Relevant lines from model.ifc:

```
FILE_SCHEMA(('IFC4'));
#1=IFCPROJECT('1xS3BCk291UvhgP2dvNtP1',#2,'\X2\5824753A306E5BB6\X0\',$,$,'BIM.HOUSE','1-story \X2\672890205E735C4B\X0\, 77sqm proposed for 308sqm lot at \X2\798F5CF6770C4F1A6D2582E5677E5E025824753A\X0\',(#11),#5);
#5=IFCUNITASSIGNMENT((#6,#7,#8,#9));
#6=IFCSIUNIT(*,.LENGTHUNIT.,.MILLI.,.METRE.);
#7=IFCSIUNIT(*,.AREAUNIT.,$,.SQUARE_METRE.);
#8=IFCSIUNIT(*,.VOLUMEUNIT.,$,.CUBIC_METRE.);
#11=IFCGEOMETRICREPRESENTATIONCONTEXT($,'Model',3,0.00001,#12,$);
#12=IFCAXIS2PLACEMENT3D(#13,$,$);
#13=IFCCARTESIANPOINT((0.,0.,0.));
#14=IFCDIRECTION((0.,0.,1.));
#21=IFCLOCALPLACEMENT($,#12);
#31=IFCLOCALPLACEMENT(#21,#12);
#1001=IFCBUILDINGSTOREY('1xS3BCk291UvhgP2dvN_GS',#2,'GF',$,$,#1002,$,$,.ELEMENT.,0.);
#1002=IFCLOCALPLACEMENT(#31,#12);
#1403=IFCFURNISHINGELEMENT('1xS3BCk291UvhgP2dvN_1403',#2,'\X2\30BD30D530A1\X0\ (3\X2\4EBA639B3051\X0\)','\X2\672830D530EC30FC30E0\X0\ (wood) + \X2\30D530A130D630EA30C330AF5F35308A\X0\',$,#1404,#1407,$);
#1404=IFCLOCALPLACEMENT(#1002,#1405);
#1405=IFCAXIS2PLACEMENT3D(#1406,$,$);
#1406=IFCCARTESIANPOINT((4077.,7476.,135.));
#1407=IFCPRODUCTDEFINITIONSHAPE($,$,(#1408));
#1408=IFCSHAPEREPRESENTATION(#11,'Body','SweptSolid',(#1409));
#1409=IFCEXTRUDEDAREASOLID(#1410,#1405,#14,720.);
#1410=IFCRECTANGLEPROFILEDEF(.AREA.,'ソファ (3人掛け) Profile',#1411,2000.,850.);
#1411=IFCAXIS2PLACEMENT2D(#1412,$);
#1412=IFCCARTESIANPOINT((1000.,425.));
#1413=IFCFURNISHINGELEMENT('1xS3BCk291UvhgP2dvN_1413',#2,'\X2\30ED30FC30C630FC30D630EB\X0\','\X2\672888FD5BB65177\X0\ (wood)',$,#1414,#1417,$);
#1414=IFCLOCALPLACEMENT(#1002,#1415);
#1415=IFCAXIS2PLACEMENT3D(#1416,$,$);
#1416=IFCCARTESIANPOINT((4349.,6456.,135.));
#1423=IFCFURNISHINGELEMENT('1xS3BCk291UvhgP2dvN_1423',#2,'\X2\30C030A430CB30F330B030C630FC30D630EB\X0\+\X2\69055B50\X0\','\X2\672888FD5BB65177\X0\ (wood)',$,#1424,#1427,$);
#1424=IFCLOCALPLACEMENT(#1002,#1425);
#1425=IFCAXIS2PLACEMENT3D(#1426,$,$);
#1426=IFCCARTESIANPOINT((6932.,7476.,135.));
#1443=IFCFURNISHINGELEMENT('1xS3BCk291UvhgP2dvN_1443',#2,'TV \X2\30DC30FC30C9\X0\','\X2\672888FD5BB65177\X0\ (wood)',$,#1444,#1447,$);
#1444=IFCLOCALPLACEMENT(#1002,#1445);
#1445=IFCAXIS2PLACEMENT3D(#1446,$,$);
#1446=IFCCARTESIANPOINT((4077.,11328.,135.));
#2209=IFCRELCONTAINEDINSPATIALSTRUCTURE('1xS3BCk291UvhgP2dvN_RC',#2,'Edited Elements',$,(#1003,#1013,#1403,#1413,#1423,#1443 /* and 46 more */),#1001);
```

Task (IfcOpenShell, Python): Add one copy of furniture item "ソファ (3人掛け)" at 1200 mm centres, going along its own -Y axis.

```python
import ifcopenshell
import ifcopenshell.api.geometry
import ifcopenshell.api.root
import ifcopenshell.util.element
import ifcopenshell.util.placement
import ifcopenshell.util.unit

model = ifcopenshell.open("model.ifc")
unit_scale = ifcopenshell.util.unit.calculate_unit_scale(model)


def reuse_history(source, copy):
    """copy_class also copies each property set's owner history, people and application; keep the originals."""
    for rel in copy.IsDefinedBy:
        if rel.is_a("IfcRelDefinesByProperties") and (history := rel.RelatingPropertyDefinition.OwnerHistory):
            rel.RelatingPropertyDefinition.OwnerHistory = source.OwnerHistory
            ifcopenshell.util.element.remove_deep2(model, history)


source = model.by_id(1403)
base = ifcopenshell.util.placement.get_local_placement(source.ObjectPlacement)
step = -base[:3, 1] * 1.2 / unit_scale

for i in range(1, 2):
    copy = ifcopenshell.api.root.copy_class(model, product=source)
    copy.Representation = ifcopenshell.util.element.copy_deep(
        model, source.Representation, exclude=["IfcGeometricRepresentationContext", "IfcRepresentationMap"]
    )
    reuse_history(source, copy)
    matrix = base.copy()
    matrix[:3, 3] += i * step
    print("added at", matrix[:3, 3].round(3) + 0.0)
    ifcopenshell.api.geometry.edit_object_placement(model, product=copy, matrix=matrix, is_si=False)

model.write("model_rev.ifc")
```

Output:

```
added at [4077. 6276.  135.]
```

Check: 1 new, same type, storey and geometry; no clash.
